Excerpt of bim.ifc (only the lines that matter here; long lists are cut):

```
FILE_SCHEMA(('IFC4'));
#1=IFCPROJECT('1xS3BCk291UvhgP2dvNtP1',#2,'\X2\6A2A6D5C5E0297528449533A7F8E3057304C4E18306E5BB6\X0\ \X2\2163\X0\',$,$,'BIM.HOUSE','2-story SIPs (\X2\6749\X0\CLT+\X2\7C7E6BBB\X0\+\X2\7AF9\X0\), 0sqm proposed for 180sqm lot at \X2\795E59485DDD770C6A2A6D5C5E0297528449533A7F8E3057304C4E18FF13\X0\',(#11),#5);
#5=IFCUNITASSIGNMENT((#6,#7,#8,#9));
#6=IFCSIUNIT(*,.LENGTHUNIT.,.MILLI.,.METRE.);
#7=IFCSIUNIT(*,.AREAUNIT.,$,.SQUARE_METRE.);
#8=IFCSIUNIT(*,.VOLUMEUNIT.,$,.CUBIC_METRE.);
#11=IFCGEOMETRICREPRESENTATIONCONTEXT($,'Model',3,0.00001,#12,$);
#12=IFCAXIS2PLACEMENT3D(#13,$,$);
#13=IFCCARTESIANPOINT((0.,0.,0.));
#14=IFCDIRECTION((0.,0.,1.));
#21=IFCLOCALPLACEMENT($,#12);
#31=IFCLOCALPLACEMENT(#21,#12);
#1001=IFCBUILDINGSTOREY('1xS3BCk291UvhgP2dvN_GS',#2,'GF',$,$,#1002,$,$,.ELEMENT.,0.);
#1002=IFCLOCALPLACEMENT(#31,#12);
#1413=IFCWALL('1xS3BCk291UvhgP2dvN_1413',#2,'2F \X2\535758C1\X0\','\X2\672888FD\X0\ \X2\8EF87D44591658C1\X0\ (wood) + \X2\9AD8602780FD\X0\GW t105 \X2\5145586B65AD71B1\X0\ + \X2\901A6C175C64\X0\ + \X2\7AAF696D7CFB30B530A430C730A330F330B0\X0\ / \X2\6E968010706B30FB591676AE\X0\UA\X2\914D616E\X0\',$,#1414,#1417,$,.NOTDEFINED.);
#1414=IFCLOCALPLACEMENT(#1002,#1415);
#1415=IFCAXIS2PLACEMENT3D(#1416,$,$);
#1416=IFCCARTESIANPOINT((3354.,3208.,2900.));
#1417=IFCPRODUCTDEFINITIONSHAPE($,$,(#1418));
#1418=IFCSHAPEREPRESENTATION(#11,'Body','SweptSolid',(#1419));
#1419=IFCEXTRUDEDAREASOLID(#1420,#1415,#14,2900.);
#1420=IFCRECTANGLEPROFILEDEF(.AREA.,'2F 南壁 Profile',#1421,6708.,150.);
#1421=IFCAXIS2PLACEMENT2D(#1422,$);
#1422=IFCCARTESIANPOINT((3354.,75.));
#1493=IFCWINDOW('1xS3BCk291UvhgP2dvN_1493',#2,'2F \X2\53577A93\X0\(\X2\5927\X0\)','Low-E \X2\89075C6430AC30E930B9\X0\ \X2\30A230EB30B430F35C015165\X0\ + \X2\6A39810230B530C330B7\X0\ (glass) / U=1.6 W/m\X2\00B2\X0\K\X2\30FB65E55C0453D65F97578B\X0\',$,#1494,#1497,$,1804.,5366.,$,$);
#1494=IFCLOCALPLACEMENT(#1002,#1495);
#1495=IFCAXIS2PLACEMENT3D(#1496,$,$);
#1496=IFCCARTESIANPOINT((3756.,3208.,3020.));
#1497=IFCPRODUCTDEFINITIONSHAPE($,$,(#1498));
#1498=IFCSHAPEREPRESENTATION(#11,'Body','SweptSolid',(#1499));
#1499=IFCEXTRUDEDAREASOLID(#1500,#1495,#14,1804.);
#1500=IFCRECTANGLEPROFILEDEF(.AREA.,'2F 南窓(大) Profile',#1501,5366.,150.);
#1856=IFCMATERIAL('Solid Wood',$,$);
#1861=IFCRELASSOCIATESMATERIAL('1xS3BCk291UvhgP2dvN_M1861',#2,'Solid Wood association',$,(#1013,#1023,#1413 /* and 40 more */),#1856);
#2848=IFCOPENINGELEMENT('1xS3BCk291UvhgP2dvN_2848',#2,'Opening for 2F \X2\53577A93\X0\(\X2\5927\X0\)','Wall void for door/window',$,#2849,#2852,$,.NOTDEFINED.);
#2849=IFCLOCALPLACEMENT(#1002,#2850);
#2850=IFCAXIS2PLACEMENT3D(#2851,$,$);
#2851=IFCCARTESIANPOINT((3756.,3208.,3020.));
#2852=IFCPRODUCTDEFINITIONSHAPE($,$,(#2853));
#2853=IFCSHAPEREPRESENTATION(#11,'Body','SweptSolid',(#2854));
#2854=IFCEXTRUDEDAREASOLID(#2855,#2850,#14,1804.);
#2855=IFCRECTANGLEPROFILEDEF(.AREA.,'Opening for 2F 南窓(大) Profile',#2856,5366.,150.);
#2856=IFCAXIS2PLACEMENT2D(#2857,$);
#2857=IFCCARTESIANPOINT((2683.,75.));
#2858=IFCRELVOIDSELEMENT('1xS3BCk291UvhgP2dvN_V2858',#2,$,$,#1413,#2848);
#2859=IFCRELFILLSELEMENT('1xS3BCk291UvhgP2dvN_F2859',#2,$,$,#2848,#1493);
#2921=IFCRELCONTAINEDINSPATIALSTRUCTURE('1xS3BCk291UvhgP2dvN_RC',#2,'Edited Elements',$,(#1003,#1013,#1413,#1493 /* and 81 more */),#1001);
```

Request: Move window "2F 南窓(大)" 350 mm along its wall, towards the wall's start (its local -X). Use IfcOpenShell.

```python
import ifcopenshell
import ifcopenshell.api.geometry
import ifcopenshell.util.placement
import ifcopenshell.util.unit

model = ifcopenshell.open("bim.ifc")
unit_scale = ifcopenshell.util.unit.calculate_unit_scale(model)

window = model.by_guid("1xS3BCk291UvhgP2dvN_1493")
opening = window.FillsVoids[0].RelatingOpeningElement
wall = opening.VoidsElements[0].RelatingBuildingElement

wall_matrix = ifcopenshell.util.placement.get_local_placement(wall.ObjectPlacement)
shift = wall_matrix[:3, 0] * -0.35 / unit_scale
before = ifcopenshell.util.placement.get_local_placement(window.ObjectPlacement)[:3, 3].copy()

# The window is not placed relative to its opening, so move both.
for product in (opening, window):
    matrix = ifcopenshell.util.placement.get_local_placement(product.ObjectPlacement)
    matrix[:3, 3] += shift
    ifcopenshell.api.geometry.edit_object_placement(model, product=product, matrix=matrix, is_si=False)

after = ifcopenshell.util.placement.get_local_placement(window.ObjectPlacement)[:3, 3]
print("window moved by", (after - before).round(3) + 0.0)

model.write("bim_updated.ifc")
```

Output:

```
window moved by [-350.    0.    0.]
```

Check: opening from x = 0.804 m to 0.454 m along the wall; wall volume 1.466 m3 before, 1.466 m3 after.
